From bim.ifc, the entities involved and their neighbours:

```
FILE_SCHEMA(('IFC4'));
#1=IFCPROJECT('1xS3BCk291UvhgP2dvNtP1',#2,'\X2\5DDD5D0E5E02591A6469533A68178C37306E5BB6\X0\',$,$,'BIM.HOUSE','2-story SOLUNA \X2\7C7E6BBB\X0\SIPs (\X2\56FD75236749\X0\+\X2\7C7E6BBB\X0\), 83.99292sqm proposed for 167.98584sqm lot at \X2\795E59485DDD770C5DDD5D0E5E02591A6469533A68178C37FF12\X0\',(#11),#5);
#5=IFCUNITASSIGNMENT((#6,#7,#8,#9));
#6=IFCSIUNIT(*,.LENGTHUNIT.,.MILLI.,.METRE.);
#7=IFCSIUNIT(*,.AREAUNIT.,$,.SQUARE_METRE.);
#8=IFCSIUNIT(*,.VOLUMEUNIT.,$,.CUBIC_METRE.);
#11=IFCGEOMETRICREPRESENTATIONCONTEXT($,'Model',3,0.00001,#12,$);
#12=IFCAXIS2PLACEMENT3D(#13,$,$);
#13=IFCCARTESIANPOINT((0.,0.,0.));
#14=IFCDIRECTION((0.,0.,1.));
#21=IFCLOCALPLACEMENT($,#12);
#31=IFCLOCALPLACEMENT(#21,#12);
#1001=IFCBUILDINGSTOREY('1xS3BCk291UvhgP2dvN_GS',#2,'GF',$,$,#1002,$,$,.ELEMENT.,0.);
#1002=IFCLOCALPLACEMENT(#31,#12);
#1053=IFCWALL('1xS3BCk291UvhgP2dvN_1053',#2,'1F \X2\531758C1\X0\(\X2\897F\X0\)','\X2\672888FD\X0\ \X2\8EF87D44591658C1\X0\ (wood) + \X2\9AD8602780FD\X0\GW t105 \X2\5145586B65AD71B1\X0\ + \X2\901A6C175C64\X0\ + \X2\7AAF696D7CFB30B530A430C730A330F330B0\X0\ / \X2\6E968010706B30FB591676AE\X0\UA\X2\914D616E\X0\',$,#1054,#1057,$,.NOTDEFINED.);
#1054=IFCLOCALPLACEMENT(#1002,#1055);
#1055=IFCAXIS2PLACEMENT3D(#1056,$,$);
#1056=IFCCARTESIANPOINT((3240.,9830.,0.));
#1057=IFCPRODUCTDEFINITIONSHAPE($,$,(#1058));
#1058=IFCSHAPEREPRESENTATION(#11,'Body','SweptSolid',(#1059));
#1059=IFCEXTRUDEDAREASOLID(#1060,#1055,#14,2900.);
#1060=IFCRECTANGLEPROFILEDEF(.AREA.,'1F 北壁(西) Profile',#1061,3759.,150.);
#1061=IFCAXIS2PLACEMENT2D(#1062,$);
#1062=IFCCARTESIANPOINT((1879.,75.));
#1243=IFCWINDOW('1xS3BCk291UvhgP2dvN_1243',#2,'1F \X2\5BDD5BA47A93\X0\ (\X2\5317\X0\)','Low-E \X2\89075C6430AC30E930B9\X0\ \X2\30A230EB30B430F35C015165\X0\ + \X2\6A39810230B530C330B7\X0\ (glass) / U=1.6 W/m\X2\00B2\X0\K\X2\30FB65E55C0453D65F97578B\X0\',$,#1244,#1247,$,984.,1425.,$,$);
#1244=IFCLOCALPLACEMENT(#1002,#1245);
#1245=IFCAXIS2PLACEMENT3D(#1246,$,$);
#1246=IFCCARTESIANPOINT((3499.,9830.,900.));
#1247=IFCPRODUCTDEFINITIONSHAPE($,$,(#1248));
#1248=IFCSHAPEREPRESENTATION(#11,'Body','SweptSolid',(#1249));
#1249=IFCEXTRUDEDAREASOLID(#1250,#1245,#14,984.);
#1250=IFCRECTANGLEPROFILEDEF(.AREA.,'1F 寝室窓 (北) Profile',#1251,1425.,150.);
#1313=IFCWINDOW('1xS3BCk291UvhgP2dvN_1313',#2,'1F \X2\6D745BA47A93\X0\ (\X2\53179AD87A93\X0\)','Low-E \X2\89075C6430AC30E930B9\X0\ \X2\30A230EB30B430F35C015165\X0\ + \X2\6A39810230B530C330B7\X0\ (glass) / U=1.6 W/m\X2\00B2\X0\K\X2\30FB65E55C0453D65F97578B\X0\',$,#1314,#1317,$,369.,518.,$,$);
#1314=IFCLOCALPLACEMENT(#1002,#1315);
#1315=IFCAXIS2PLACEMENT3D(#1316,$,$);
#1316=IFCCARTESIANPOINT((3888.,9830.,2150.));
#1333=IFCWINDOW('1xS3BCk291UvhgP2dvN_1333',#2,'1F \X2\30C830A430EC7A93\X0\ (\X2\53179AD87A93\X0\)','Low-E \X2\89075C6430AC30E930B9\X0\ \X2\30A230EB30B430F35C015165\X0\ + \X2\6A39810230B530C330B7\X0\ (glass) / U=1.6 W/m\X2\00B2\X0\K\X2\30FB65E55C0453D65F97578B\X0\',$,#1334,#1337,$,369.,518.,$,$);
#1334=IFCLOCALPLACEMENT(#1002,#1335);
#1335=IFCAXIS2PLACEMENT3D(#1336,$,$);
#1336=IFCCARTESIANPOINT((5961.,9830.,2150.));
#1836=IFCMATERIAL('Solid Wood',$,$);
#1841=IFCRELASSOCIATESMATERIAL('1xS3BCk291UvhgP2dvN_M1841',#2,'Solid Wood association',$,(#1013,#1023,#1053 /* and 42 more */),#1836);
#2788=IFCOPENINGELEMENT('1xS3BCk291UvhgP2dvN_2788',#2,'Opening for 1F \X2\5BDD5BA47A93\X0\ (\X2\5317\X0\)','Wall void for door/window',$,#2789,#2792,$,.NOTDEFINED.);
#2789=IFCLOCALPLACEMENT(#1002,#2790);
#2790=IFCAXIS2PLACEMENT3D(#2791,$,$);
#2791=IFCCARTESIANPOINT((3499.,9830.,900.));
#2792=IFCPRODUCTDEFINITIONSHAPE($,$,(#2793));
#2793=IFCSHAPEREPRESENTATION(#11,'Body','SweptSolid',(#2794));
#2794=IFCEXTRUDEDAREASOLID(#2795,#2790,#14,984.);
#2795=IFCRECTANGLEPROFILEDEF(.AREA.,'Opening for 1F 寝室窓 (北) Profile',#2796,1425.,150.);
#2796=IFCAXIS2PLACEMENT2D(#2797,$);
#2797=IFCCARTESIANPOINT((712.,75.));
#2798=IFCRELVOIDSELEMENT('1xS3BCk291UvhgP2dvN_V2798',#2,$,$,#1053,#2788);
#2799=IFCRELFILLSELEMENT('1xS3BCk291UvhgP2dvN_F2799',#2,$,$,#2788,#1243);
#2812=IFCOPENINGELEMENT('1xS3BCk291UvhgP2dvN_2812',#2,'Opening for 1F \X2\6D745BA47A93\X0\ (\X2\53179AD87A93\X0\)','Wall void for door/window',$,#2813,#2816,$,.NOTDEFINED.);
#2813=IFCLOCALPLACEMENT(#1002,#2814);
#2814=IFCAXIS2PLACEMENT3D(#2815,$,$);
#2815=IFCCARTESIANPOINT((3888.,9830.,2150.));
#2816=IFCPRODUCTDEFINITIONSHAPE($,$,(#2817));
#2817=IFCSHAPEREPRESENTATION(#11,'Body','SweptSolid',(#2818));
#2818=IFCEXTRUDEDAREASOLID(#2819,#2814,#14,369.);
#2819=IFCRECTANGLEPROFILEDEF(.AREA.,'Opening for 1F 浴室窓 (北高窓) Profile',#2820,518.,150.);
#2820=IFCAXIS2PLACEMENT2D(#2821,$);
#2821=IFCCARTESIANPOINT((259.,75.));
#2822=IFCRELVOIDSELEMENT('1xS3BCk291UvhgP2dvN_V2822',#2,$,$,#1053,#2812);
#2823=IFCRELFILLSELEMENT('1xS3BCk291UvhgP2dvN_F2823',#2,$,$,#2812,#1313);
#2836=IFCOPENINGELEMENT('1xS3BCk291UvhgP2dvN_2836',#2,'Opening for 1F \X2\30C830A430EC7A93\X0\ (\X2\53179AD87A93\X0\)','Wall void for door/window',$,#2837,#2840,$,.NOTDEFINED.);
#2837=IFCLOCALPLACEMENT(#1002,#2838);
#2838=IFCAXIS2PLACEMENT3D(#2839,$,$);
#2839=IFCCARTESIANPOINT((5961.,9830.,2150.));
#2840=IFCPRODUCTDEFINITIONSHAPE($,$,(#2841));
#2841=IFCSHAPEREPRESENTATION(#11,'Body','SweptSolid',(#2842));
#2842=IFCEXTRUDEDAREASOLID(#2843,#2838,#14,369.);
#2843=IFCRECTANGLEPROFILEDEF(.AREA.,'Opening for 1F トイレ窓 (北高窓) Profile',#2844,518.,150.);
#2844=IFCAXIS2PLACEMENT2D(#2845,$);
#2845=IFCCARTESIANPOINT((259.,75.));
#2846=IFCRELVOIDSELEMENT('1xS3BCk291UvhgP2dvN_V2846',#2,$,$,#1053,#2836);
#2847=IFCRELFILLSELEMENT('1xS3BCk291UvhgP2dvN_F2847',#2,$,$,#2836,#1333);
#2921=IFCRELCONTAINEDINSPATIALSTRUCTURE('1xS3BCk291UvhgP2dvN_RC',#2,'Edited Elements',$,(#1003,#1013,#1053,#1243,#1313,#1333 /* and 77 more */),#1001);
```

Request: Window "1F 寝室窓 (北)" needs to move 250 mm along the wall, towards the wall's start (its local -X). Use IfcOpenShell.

```python
import ifcopenshell
import ifcopenshell.api.geometry
import ifcopenshell.util.placement
import ifcopenshell.util.unit

model = ifcopenshell.open("bim.ifc")
unit_scale = ifcopenshell.util.unit.calculate_unit_scale(model)

window = model.by_guid("1xS3BCk291UvhgP2dvN_1243")
opening = window.FillsVoids[0].RelatingOpeningElement
wall = opening.VoidsElements[0].RelatingBuildingElement

wall_matrix = ifcopenshell.util.placement.get_local_placement(wall.ObjectPlacement)
shift = wall_matrix[:3, 0] * -0.25 / unit_scale
before = ifcopenshell.util.placement.get_local_placement(window.ObjectPlacement)[:3, 3].copy()

# The window is not placed relative to its opening, so move both.
for product in (opening, window):
    matrix = ifcopenshell.util.placement.get_local_placement(product.ObjectPlacement)
    matrix[:3, 3] += shift
    ifcopenshell.api.geometry.edit_object_placement(model, product=product, matrix=matrix, is_si=False)

after = ifcopenshell.util.placement.get_local_placement(window.ObjectPlacement)[:3, 3]
print("window moved by", (after - before).round(3) + 0.0)

model.write("bim_edited.ifc")
```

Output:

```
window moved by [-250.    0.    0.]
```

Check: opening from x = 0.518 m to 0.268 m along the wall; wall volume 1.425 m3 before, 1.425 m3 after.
